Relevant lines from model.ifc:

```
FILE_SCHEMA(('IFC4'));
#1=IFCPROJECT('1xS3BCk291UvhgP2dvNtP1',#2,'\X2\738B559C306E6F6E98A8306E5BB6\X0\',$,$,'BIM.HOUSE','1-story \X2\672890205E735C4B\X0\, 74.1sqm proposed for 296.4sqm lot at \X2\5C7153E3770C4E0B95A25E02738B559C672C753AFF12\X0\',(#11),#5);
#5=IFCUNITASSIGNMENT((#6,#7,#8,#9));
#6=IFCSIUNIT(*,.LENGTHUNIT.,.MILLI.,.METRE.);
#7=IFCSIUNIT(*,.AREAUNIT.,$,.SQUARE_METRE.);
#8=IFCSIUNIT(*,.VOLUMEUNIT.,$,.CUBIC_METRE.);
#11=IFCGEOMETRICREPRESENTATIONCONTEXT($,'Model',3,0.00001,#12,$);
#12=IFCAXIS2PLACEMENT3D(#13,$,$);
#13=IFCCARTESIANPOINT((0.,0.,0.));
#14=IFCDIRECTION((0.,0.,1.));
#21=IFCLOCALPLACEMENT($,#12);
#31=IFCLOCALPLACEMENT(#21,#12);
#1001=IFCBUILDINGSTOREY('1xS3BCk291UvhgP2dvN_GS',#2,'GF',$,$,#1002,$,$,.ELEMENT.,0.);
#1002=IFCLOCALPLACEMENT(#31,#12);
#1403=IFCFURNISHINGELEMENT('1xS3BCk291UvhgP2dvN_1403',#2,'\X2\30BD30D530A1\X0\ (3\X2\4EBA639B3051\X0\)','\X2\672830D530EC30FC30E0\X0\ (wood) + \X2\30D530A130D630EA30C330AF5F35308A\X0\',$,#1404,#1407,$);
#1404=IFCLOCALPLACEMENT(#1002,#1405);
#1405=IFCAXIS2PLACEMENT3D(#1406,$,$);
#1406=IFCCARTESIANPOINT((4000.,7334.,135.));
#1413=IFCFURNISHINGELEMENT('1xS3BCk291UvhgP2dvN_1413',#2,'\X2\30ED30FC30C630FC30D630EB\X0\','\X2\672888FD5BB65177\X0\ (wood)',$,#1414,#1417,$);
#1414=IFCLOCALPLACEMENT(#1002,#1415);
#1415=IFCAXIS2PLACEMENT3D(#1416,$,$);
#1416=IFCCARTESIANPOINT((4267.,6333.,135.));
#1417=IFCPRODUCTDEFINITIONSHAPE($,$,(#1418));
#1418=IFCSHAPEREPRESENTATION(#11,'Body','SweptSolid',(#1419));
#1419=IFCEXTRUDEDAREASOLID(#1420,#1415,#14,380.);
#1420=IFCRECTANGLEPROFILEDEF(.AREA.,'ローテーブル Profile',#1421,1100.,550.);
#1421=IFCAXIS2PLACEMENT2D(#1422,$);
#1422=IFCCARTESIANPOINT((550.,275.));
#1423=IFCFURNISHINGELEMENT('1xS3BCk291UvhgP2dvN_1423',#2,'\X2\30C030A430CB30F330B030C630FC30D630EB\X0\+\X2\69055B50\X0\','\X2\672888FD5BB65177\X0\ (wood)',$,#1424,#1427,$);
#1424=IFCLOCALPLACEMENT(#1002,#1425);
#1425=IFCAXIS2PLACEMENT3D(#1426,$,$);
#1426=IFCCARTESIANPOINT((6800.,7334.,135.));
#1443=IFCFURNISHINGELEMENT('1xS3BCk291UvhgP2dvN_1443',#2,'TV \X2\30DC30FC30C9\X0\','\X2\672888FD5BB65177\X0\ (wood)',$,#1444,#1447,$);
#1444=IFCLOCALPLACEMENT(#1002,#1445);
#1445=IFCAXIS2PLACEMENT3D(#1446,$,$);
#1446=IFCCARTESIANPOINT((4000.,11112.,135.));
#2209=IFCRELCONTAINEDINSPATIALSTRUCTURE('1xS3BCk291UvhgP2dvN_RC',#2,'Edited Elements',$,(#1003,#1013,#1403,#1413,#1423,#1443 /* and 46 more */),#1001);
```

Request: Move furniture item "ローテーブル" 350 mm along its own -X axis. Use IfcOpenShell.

```python
import ifcopenshell
import ifcopenshell.api.geometry
import ifcopenshell.util.placement

model = ifcopenshell.open("model.ifc")

item = model.by_id(1413)
matrix = ifcopenshell.util.placement.get_local_placement(item.ObjectPlacement)
matrix[:3, 3] -= matrix[:3, 0] * 350.0
ifcopenshell.api.geometry.edit_object_placement(model, product=item, matrix=matrix, is_si=False)

print(ifcopenshell.util.placement.get_local_placement(item.ObjectPlacement).round(3) + 0.0)

model.write("model_v2.ifc")
```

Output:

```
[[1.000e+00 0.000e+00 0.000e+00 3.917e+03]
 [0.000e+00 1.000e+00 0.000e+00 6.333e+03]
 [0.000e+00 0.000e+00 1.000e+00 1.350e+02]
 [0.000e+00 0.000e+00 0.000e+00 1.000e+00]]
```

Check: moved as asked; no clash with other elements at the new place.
